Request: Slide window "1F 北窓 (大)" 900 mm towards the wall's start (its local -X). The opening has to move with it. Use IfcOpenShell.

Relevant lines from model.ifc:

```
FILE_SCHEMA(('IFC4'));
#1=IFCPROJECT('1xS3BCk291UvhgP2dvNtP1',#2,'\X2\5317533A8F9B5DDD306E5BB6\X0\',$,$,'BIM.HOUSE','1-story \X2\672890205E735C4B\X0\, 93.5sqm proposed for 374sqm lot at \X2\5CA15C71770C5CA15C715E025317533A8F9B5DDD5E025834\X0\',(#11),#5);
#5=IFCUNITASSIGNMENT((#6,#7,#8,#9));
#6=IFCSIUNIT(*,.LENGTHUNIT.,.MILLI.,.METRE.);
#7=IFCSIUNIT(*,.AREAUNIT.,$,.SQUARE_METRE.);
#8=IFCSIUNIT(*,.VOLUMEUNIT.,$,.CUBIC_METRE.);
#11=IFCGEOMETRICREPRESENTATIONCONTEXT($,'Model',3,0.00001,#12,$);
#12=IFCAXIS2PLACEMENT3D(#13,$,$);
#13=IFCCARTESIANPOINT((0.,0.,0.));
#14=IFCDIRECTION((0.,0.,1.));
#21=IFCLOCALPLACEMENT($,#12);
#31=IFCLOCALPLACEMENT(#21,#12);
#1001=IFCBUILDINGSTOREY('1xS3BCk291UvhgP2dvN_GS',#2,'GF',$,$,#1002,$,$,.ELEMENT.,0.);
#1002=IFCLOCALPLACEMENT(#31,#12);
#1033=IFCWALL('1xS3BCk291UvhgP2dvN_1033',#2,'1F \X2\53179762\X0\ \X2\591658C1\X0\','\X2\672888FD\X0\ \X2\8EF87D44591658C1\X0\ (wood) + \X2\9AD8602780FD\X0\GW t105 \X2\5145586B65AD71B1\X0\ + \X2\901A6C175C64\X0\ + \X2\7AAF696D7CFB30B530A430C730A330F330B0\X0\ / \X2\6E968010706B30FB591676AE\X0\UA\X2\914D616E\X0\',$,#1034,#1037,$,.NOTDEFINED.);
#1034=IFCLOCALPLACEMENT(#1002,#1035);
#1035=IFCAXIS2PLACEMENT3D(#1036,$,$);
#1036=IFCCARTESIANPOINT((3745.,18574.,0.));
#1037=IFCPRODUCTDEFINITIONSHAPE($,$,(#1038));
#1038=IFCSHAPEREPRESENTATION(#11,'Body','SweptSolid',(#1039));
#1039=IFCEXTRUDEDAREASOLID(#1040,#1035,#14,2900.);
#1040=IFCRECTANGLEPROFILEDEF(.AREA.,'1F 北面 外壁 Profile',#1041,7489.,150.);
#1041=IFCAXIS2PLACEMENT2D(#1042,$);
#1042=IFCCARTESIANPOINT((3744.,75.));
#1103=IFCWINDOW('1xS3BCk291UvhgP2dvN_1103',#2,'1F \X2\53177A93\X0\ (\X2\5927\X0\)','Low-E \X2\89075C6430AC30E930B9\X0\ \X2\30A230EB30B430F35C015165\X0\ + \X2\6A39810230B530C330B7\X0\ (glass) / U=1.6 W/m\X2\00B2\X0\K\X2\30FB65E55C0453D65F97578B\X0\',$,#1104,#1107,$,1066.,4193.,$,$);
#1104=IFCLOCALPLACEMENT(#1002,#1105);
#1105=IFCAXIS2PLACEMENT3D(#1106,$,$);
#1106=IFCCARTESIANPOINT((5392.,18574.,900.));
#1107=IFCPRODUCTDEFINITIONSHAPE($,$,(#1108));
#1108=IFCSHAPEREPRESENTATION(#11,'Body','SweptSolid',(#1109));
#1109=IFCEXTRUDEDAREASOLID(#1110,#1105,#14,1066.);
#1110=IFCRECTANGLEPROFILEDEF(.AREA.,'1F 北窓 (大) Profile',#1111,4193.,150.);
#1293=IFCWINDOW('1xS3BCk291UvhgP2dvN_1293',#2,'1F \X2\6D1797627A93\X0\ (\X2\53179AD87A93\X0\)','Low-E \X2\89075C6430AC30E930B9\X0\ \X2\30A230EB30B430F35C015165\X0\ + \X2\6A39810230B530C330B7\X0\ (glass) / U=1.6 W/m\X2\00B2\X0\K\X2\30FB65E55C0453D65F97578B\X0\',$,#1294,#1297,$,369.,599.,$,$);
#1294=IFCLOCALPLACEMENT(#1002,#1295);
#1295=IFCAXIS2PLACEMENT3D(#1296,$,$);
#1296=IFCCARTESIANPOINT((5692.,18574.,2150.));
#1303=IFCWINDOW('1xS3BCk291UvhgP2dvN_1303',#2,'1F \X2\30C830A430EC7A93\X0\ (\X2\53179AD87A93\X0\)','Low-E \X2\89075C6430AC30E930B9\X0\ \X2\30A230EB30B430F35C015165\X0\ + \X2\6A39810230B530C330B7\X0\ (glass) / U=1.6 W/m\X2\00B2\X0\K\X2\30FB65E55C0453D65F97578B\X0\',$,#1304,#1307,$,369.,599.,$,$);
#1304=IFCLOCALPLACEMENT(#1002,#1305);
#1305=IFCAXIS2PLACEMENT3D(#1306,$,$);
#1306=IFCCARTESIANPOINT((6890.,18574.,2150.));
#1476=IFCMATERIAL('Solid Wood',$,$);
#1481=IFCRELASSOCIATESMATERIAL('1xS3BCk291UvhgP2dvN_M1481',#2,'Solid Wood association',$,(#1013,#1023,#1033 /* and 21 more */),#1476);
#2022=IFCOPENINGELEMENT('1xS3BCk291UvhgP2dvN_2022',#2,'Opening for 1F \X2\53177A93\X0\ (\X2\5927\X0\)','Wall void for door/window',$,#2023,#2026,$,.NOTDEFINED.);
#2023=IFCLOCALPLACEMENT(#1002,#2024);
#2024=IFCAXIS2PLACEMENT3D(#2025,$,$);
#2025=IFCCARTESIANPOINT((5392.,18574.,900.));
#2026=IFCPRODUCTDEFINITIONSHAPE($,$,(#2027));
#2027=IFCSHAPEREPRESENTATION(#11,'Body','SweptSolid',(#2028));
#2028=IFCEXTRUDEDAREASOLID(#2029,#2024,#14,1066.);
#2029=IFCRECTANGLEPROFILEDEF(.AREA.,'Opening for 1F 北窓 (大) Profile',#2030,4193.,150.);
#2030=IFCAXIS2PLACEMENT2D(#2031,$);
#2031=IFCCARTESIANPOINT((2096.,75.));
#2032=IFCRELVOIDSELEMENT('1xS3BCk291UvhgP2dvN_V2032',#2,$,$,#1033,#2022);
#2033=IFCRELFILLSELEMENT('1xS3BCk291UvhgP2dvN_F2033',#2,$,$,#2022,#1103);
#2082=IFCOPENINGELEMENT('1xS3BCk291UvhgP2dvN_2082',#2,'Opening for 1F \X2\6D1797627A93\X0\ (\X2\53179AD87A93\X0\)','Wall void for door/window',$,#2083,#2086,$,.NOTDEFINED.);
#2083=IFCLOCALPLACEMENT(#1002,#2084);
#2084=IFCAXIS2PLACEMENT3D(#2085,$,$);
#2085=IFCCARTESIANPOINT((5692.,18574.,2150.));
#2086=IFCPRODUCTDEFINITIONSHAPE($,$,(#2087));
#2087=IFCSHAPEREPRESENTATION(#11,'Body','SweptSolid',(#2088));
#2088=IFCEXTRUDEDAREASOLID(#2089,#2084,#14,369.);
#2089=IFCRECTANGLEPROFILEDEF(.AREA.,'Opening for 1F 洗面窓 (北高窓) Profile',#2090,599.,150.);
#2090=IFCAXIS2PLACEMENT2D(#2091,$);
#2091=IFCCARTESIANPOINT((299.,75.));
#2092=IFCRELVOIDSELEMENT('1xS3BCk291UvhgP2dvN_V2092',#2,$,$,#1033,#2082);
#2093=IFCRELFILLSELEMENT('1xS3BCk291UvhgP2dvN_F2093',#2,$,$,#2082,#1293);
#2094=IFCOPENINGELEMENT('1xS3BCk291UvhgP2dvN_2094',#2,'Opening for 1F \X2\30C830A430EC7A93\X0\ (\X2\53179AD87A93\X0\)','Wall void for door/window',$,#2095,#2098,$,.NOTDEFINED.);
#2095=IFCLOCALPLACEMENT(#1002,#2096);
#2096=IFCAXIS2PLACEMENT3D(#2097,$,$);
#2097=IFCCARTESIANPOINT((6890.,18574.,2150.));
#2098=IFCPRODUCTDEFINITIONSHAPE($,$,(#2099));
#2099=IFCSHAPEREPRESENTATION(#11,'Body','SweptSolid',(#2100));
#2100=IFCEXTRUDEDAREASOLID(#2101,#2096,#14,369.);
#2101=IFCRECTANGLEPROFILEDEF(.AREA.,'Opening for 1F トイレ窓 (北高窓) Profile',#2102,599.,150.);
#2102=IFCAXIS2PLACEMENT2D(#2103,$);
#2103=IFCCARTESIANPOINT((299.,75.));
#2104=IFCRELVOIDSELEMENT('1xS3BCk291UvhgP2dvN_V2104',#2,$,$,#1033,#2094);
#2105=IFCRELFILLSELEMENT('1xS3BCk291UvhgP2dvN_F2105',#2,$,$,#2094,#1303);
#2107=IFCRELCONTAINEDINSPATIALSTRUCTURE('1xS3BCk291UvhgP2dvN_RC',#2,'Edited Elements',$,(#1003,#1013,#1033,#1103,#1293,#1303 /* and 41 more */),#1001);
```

```python
import ifcopenshell
import ifcopenshell.api.geometry
import ifcopenshell.util.placement

model = ifcopenshell.open("model.ifc")

window = model.by_guid("1xS3BCk291UvhgP2dvN_1103")
opening = window.FillsVoids[0].RelatingOpeningElement
wall = opening.VoidsElements[0].RelatingBuildingElement

wall_matrix = ifcopenshell.util.placement.get_local_placement(wall.ObjectPlacement)
shift = wall_matrix[:3, 0] * -900.0
before = ifcopenshell.util.placement.get_local_placement(window.ObjectPlacement)[:3, 3].copy()

# The window is not placed relative to its opening, so move both.
for product in (opening, window):
    matrix = ifcopenshell.util.placement.get_local_placement(product.ObjectPlacement)
    matrix[:3, 3] += shift
    ifcopenshell.api.geometry.edit_object_placement(model, product=product, matrix=matrix, is_si=False)

after = ifcopenshell.util.placement.get_local_placement(window.ObjectPlacement)[:3, 3]
print("window moved by", (after - before).round(3) + 0.0)

model.write("model_updated.ifc")
```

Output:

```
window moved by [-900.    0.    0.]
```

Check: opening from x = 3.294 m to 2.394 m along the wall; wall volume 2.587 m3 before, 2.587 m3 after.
